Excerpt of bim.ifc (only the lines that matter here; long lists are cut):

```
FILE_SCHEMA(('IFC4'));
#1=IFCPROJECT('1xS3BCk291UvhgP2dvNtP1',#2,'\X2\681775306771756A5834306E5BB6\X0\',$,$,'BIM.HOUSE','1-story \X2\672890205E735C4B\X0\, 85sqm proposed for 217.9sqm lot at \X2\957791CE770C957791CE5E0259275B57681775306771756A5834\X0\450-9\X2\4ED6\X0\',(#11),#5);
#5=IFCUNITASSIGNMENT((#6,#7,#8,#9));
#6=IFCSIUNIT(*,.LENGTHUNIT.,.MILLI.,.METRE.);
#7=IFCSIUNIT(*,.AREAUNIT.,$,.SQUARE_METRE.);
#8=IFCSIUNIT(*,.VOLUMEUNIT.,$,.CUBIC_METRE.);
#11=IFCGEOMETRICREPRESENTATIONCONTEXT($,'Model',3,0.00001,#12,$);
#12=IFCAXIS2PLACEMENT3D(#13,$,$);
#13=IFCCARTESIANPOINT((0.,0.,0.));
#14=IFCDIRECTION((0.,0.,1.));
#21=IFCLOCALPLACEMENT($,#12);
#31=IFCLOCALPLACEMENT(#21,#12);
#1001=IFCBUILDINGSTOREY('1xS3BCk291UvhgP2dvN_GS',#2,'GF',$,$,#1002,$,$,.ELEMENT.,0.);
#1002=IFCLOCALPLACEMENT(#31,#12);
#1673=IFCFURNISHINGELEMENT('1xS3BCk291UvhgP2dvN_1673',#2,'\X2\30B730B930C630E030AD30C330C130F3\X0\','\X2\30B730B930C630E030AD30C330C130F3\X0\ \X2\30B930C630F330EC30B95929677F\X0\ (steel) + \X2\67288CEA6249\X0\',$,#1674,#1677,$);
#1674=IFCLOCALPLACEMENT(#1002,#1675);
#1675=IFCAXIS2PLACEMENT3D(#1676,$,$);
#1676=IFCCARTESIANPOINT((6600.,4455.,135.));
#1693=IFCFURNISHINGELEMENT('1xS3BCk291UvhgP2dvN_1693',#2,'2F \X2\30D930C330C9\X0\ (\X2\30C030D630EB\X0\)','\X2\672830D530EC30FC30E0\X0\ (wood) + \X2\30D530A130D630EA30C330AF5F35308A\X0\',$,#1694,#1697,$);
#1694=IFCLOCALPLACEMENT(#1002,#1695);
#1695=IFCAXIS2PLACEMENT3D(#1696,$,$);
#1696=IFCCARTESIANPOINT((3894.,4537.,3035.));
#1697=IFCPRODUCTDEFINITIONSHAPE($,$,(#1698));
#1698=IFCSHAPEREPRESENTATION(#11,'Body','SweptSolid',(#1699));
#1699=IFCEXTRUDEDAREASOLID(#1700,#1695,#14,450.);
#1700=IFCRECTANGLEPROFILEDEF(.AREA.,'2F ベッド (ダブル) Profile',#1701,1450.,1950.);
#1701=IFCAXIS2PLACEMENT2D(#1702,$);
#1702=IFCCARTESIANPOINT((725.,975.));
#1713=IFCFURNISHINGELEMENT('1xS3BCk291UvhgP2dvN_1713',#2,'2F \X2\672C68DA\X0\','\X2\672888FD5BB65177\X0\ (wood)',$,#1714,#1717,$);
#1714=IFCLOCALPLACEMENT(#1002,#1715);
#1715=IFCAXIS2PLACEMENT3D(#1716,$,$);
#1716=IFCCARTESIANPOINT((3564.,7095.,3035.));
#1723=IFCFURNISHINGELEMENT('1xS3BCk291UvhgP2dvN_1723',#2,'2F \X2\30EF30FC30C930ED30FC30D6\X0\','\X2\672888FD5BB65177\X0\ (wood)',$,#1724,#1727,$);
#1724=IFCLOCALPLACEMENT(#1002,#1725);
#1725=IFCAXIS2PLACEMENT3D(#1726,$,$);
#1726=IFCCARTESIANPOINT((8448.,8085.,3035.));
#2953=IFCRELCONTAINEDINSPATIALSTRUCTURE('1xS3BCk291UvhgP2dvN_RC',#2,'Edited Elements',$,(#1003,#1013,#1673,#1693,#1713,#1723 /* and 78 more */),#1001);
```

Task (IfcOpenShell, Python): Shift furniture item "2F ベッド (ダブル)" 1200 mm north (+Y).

```python
import ifcopenshell
import ifcopenshell.api.geometry
import ifcopenshell.util.placement

model = ifcopenshell.open("bim.ifc")

item = model.by_guid("1xS3BCk291UvhgP2dvN_1693")
matrix = ifcopenshell.util.placement.get_local_placement(item.ObjectPlacement)
matrix[1, 3] += 1200.0
ifcopenshell.api.geometry.edit_object_placement(model, product=item, matrix=matrix, is_si=False)

print(ifcopenshell.util.placement.get_local_placement(item.ObjectPlacement).round(3) + 0.0)

model.write("bim-out.ifc")
```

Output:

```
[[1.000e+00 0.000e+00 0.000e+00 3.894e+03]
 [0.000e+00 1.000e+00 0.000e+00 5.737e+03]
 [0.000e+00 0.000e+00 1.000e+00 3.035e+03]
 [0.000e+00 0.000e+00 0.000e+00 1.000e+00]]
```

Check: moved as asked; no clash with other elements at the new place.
